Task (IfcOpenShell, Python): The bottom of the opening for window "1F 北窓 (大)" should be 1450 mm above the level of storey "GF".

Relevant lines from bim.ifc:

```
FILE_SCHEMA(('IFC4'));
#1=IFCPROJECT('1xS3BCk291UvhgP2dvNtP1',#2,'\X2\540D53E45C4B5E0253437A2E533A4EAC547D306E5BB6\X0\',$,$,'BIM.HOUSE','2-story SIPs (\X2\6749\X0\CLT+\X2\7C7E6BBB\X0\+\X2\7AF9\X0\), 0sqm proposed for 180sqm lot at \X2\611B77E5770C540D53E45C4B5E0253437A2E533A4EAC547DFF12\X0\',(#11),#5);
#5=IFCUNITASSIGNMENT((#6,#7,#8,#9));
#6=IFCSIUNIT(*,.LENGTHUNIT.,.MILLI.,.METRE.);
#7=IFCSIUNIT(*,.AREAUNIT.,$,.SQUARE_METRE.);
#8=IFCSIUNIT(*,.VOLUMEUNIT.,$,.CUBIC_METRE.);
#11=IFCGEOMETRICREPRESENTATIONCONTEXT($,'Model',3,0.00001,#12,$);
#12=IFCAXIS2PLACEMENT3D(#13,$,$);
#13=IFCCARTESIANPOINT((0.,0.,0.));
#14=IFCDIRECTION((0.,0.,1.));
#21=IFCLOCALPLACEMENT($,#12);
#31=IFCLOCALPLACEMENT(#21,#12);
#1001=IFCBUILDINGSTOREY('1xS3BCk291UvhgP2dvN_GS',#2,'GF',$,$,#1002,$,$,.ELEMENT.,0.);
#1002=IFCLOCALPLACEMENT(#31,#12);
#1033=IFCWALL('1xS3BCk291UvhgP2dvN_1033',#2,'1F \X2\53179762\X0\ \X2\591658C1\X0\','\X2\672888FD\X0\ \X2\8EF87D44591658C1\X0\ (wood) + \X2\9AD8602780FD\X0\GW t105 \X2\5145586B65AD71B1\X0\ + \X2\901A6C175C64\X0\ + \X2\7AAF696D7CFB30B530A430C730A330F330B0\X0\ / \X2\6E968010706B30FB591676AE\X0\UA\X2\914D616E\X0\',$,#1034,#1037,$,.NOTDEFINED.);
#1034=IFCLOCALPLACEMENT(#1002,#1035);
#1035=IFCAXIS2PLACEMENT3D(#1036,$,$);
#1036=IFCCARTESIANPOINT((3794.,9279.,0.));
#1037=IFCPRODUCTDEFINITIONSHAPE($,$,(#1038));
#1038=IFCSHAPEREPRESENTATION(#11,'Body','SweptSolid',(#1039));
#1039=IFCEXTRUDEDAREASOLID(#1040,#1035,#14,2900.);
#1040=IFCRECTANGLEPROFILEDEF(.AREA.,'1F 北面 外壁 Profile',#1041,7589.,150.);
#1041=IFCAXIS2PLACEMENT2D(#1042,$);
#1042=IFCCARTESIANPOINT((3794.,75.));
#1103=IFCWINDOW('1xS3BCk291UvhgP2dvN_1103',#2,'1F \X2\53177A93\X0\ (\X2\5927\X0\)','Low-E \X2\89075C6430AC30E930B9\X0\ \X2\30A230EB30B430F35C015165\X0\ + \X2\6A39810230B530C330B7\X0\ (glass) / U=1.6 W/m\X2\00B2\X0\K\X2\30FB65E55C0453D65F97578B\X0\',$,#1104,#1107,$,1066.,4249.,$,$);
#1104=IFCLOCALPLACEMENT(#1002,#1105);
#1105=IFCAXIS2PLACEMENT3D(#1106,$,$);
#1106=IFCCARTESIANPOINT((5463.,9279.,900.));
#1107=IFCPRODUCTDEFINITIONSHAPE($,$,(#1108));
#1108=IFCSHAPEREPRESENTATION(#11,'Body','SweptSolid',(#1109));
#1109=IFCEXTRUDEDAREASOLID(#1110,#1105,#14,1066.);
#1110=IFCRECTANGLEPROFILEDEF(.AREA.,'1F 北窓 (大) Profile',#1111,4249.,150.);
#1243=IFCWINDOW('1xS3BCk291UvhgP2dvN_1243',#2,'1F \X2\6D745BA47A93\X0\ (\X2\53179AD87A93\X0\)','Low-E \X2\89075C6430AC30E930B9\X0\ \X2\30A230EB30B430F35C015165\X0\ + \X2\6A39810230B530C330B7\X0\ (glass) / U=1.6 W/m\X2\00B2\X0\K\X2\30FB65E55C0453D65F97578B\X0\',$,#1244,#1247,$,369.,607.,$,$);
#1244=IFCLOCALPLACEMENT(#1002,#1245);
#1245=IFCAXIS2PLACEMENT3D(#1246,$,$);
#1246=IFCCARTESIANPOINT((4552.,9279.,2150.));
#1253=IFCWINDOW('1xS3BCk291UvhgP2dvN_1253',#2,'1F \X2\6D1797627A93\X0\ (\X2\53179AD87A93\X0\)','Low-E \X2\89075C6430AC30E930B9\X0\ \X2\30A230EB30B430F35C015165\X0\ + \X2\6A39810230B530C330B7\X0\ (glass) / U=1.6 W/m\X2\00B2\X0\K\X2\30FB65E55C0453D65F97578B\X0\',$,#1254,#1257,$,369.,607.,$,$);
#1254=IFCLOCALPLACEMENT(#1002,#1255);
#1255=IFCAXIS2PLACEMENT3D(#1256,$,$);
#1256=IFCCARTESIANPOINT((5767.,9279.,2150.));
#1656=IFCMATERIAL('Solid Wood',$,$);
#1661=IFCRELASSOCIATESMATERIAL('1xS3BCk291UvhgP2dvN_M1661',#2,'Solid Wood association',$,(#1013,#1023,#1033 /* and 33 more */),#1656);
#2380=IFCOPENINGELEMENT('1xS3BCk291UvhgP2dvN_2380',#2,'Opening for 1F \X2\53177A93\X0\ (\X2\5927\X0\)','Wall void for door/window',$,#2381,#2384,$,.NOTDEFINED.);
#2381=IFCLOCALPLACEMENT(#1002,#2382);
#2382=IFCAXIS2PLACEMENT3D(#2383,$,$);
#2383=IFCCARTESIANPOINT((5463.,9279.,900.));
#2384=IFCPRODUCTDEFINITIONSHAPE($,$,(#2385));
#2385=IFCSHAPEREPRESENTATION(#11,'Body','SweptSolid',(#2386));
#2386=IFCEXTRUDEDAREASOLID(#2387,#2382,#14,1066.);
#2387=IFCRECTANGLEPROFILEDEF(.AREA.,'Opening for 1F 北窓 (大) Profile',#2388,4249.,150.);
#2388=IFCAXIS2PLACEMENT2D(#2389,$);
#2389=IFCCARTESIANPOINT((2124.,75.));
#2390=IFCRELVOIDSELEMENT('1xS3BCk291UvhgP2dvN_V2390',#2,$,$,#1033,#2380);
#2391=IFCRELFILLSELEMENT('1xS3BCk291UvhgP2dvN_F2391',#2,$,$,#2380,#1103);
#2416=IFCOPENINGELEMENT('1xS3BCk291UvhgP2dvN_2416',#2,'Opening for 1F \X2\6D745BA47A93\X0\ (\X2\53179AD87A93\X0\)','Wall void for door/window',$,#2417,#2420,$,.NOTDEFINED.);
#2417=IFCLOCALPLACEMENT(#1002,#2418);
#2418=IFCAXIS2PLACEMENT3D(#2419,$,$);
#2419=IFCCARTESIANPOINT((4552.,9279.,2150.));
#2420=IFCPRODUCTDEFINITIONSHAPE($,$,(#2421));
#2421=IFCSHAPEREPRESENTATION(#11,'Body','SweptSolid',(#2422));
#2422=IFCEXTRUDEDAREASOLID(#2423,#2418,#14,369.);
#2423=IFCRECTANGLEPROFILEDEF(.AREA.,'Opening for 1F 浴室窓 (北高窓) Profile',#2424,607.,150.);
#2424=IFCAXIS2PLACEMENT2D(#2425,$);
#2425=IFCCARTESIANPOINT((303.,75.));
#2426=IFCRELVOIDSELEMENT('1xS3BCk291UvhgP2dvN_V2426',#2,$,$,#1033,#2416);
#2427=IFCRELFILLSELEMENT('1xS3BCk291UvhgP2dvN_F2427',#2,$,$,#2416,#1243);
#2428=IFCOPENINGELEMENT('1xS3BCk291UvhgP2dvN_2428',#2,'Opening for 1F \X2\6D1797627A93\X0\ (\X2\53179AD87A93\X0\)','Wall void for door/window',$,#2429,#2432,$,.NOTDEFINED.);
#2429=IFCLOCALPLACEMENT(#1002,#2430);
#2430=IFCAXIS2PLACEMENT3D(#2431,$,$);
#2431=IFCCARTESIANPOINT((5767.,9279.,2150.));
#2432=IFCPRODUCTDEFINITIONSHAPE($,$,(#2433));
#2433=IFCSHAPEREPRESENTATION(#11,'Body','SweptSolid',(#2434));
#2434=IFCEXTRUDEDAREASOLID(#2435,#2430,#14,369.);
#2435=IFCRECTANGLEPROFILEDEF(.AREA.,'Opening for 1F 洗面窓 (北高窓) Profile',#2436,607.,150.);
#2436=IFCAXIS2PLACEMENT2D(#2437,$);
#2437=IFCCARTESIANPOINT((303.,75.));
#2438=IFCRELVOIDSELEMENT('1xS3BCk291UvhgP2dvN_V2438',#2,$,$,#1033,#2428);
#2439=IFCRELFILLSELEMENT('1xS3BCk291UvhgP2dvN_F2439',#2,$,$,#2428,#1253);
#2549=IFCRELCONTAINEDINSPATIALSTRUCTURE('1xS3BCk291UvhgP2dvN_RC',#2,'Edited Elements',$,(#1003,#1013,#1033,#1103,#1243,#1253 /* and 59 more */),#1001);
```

```python
import numpy as np
import ifcopenshell
import ifcopenshell.api.geometry
import ifcopenshell.geom
import ifcopenshell.util.element
import ifcopenshell.util.placement
import ifcopenshell.util.shape
import ifcopenshell.util.unit

model = ifcopenshell.open("bim.ifc")
unit_scale = ifcopenshell.util.unit.calculate_unit_scale(model)

window = model.by_id(1103)
opening = window.FillsVoids[0].RelatingOpeningElement
storey = ifcopenshell.util.element.get_container(window, ifc_class="IfcBuildingStorey")
level = ifcopenshell.util.placement.get_local_placement(storey.ObjectPlacement)[2, 3]

# The opening's origin need not be at the sill, so measure its lowest point.
shape = ifcopenshell.geom.create_shape(ifcopenshell.geom.settings(), opening)
bottom = ifcopenshell.util.shape.get_shape_bottom_elevation(shape, shape.geometry) / unit_scale
dz = level + 1450.0 - bottom

shift = np.array([0.0, 0.0, dz])
# The window is not placed relative to its opening, so move both.
for product in (opening, window):
    matrix = ifcopenshell.util.placement.get_local_placement(product.ObjectPlacement)
    matrix[:3, 3] += shift
    ifcopenshell.api.geometry.edit_object_placement(model, product=product, matrix=matrix, is_si=False)

print(f"moved by {dz * unit_scale:+.3f} m")

model.write("bim_updated.ifc")
```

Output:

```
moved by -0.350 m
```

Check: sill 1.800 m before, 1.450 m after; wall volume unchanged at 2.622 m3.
